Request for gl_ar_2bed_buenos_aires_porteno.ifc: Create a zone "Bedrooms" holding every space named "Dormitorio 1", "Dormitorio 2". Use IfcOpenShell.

First a look at what the model holds.

```python
import ifcopenshell

model = ifcopenshell.open("gl_ar_2bed_buenos_aires_porteno.ifc")
print(model.schema)
seen = {}
for space in model.by_type("IfcSpace"):
    seen[space.LongName] = seen.get(space.LongName, 0) + 1
for name, count in sorted(seen.items(), key=str):
    print(count, "x", name)
print("zones:", [z.Name for z in model.by_type("IfcZone")][:20])
```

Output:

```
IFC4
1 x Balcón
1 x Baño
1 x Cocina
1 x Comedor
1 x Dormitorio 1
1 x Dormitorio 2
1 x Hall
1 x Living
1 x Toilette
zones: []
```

```python
import ifcopenshell
import ifcopenshell.api.group
import ifcopenshell.api.root

model = ifcopenshell.open("gl_ar_2bed_buenos_aires_porteno.ifc")

names = {"Dormitorio 1", "Dormitorio 2"}
spaces = [s for s in model.by_type("IfcSpace") if s.LongName in names]

zone = ifcopenshell.api.root.create_entity(model, ifc_class="IfcZone", name="Bedrooms")
ifcopenshell.api.group.assign_group(model, products=spaces, group=zone)
print(len(spaces), "spaces in", zone.Name)

model.write("gl_ar_2bed_buenos_aires_porteno_edited.ifc")
```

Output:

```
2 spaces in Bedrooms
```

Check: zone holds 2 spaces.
